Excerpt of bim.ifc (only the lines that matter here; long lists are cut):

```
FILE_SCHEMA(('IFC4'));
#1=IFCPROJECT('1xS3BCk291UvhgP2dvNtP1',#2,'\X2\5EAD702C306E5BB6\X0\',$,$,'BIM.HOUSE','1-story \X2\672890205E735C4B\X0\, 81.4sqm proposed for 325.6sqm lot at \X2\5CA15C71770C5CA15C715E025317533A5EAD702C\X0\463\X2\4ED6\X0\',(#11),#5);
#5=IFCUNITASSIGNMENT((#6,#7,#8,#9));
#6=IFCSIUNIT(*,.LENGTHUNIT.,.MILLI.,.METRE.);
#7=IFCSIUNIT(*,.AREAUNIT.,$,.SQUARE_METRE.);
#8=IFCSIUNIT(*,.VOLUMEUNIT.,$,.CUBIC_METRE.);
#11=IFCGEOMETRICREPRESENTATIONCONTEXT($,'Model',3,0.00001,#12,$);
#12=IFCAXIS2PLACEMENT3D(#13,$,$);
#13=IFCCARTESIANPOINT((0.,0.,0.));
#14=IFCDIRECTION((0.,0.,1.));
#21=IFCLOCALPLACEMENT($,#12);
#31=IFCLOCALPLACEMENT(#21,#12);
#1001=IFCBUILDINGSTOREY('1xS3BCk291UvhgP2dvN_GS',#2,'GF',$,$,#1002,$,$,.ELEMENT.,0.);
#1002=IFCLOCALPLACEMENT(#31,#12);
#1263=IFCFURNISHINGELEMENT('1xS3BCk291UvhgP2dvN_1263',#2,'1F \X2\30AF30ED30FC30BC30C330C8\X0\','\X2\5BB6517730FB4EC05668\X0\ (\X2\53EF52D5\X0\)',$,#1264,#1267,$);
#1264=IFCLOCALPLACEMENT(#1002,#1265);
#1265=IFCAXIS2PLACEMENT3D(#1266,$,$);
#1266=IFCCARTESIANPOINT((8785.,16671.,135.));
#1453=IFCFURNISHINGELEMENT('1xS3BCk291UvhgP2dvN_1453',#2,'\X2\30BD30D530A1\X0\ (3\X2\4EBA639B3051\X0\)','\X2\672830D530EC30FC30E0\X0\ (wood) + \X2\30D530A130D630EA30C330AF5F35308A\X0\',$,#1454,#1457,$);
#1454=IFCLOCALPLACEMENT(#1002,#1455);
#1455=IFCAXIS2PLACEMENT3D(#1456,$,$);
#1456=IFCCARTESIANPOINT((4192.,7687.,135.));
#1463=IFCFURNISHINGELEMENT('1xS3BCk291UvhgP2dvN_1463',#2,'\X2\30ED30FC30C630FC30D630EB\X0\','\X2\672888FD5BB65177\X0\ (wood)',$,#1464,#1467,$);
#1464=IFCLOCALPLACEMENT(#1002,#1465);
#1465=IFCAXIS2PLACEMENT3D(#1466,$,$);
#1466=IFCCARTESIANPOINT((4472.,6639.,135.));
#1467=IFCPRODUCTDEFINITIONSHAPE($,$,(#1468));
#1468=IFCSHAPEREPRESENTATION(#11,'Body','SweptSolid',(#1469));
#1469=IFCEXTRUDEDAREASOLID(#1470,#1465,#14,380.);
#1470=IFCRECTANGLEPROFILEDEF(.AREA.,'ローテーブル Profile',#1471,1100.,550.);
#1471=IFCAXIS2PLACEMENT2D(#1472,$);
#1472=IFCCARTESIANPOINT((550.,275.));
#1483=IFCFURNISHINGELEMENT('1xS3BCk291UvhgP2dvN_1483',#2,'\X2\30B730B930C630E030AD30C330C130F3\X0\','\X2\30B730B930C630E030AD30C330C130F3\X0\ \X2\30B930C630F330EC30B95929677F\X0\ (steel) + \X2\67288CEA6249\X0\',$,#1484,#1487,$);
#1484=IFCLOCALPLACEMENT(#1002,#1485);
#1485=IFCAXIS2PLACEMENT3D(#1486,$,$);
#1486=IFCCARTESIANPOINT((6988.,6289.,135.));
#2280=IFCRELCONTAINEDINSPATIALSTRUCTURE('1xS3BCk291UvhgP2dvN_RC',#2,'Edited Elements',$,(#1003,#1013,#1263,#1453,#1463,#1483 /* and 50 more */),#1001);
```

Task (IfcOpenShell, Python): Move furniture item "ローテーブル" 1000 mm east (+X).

```python
import ifcopenshell
import ifcopenshell.api.geometry
import ifcopenshell.util.placement
import ifcopenshell.util.unit

model = ifcopenshell.open("bim.ifc")
unit_scale = ifcopenshell.util.unit.calculate_unit_scale(model)

item = model.by_id(1463)
matrix = ifcopenshell.util.placement.get_local_placement(item.ObjectPlacement)
matrix[0, 3] += 1 / unit_scale
ifcopenshell.api.geometry.edit_object_placement(model, product=item, matrix=matrix, is_si=False)

print(ifcopenshell.util.placement.get_local_placement(item.ObjectPlacement).round(3) + 0.0)

model.write("bim_updated.ifc")
```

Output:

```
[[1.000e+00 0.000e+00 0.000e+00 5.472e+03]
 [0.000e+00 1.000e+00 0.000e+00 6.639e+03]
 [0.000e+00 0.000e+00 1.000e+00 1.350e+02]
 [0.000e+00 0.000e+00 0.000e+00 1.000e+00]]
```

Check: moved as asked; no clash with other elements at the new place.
